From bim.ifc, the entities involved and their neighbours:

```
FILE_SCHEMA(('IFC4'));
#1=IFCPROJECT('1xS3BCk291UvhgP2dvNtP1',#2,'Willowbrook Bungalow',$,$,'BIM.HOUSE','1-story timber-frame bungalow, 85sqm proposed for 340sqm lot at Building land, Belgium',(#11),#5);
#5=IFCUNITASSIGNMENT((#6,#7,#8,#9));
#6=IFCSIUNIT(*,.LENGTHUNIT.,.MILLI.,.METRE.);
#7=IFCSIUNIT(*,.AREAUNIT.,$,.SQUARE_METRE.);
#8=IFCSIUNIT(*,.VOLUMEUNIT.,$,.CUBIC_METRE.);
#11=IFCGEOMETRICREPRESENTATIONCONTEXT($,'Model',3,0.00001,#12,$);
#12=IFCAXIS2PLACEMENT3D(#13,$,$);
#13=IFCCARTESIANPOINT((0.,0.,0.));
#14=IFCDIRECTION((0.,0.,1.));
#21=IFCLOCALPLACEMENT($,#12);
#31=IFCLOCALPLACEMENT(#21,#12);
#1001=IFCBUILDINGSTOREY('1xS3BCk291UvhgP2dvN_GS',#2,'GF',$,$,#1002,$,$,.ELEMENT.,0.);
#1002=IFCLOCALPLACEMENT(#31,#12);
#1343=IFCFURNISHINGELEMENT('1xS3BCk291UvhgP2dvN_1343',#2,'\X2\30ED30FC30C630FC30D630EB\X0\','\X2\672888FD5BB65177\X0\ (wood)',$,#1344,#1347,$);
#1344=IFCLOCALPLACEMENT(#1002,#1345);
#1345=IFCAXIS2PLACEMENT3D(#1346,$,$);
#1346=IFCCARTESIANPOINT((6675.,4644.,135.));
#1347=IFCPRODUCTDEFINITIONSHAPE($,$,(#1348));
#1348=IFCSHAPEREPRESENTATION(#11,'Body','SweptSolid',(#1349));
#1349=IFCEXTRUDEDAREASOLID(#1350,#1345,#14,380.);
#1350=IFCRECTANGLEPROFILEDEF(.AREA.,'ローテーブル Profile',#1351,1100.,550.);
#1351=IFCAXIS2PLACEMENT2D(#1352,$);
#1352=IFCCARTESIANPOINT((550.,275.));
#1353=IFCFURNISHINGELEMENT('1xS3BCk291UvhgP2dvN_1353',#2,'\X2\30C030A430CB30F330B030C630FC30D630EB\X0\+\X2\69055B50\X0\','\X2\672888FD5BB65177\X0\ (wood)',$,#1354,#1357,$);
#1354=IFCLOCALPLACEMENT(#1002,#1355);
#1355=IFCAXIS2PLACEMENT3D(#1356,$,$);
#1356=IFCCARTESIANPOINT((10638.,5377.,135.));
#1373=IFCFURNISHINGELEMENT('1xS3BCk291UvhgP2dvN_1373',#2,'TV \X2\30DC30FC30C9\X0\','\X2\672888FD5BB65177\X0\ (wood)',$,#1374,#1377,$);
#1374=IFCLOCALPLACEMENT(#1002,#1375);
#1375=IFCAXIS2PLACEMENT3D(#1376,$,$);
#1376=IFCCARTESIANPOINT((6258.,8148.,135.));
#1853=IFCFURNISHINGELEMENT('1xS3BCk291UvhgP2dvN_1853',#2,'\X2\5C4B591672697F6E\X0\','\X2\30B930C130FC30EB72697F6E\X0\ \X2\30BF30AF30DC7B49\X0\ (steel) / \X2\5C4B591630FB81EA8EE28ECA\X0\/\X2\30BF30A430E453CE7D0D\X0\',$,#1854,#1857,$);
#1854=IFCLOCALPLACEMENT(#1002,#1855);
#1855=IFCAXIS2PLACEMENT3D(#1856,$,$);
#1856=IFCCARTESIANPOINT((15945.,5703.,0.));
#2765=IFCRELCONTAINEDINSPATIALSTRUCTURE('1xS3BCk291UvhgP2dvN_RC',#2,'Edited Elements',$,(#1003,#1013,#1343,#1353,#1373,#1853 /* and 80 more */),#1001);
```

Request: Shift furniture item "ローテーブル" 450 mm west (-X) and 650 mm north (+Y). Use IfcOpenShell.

```python
import ifcopenshell
import ifcopenshell.api.geometry
import ifcopenshell.util.placement
import ifcopenshell.util.unit

model = ifcopenshell.open("bim.ifc")
unit_scale = ifcopenshell.util.unit.calculate_unit_scale(model)

item = model.by_guid("1xS3BCk291UvhgP2dvN_1343")
matrix = ifcopenshell.util.placement.get_local_placement(item.ObjectPlacement)
matrix[0, 3] -= 0.45 / unit_scale
matrix[1, 3] += 0.65 / unit_scale
ifcopenshell.api.geometry.edit_object_placement(model, product=item, matrix=matrix, is_si=False)

print(ifcopenshell.util.placement.get_local_placement(item.ObjectPlacement).round(3) + 0.0)

model.write("bim_updated.ifc")
```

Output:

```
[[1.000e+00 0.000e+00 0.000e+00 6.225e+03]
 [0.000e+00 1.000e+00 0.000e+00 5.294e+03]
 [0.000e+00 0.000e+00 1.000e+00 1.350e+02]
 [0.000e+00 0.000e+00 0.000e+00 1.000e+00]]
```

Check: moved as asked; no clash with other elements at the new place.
